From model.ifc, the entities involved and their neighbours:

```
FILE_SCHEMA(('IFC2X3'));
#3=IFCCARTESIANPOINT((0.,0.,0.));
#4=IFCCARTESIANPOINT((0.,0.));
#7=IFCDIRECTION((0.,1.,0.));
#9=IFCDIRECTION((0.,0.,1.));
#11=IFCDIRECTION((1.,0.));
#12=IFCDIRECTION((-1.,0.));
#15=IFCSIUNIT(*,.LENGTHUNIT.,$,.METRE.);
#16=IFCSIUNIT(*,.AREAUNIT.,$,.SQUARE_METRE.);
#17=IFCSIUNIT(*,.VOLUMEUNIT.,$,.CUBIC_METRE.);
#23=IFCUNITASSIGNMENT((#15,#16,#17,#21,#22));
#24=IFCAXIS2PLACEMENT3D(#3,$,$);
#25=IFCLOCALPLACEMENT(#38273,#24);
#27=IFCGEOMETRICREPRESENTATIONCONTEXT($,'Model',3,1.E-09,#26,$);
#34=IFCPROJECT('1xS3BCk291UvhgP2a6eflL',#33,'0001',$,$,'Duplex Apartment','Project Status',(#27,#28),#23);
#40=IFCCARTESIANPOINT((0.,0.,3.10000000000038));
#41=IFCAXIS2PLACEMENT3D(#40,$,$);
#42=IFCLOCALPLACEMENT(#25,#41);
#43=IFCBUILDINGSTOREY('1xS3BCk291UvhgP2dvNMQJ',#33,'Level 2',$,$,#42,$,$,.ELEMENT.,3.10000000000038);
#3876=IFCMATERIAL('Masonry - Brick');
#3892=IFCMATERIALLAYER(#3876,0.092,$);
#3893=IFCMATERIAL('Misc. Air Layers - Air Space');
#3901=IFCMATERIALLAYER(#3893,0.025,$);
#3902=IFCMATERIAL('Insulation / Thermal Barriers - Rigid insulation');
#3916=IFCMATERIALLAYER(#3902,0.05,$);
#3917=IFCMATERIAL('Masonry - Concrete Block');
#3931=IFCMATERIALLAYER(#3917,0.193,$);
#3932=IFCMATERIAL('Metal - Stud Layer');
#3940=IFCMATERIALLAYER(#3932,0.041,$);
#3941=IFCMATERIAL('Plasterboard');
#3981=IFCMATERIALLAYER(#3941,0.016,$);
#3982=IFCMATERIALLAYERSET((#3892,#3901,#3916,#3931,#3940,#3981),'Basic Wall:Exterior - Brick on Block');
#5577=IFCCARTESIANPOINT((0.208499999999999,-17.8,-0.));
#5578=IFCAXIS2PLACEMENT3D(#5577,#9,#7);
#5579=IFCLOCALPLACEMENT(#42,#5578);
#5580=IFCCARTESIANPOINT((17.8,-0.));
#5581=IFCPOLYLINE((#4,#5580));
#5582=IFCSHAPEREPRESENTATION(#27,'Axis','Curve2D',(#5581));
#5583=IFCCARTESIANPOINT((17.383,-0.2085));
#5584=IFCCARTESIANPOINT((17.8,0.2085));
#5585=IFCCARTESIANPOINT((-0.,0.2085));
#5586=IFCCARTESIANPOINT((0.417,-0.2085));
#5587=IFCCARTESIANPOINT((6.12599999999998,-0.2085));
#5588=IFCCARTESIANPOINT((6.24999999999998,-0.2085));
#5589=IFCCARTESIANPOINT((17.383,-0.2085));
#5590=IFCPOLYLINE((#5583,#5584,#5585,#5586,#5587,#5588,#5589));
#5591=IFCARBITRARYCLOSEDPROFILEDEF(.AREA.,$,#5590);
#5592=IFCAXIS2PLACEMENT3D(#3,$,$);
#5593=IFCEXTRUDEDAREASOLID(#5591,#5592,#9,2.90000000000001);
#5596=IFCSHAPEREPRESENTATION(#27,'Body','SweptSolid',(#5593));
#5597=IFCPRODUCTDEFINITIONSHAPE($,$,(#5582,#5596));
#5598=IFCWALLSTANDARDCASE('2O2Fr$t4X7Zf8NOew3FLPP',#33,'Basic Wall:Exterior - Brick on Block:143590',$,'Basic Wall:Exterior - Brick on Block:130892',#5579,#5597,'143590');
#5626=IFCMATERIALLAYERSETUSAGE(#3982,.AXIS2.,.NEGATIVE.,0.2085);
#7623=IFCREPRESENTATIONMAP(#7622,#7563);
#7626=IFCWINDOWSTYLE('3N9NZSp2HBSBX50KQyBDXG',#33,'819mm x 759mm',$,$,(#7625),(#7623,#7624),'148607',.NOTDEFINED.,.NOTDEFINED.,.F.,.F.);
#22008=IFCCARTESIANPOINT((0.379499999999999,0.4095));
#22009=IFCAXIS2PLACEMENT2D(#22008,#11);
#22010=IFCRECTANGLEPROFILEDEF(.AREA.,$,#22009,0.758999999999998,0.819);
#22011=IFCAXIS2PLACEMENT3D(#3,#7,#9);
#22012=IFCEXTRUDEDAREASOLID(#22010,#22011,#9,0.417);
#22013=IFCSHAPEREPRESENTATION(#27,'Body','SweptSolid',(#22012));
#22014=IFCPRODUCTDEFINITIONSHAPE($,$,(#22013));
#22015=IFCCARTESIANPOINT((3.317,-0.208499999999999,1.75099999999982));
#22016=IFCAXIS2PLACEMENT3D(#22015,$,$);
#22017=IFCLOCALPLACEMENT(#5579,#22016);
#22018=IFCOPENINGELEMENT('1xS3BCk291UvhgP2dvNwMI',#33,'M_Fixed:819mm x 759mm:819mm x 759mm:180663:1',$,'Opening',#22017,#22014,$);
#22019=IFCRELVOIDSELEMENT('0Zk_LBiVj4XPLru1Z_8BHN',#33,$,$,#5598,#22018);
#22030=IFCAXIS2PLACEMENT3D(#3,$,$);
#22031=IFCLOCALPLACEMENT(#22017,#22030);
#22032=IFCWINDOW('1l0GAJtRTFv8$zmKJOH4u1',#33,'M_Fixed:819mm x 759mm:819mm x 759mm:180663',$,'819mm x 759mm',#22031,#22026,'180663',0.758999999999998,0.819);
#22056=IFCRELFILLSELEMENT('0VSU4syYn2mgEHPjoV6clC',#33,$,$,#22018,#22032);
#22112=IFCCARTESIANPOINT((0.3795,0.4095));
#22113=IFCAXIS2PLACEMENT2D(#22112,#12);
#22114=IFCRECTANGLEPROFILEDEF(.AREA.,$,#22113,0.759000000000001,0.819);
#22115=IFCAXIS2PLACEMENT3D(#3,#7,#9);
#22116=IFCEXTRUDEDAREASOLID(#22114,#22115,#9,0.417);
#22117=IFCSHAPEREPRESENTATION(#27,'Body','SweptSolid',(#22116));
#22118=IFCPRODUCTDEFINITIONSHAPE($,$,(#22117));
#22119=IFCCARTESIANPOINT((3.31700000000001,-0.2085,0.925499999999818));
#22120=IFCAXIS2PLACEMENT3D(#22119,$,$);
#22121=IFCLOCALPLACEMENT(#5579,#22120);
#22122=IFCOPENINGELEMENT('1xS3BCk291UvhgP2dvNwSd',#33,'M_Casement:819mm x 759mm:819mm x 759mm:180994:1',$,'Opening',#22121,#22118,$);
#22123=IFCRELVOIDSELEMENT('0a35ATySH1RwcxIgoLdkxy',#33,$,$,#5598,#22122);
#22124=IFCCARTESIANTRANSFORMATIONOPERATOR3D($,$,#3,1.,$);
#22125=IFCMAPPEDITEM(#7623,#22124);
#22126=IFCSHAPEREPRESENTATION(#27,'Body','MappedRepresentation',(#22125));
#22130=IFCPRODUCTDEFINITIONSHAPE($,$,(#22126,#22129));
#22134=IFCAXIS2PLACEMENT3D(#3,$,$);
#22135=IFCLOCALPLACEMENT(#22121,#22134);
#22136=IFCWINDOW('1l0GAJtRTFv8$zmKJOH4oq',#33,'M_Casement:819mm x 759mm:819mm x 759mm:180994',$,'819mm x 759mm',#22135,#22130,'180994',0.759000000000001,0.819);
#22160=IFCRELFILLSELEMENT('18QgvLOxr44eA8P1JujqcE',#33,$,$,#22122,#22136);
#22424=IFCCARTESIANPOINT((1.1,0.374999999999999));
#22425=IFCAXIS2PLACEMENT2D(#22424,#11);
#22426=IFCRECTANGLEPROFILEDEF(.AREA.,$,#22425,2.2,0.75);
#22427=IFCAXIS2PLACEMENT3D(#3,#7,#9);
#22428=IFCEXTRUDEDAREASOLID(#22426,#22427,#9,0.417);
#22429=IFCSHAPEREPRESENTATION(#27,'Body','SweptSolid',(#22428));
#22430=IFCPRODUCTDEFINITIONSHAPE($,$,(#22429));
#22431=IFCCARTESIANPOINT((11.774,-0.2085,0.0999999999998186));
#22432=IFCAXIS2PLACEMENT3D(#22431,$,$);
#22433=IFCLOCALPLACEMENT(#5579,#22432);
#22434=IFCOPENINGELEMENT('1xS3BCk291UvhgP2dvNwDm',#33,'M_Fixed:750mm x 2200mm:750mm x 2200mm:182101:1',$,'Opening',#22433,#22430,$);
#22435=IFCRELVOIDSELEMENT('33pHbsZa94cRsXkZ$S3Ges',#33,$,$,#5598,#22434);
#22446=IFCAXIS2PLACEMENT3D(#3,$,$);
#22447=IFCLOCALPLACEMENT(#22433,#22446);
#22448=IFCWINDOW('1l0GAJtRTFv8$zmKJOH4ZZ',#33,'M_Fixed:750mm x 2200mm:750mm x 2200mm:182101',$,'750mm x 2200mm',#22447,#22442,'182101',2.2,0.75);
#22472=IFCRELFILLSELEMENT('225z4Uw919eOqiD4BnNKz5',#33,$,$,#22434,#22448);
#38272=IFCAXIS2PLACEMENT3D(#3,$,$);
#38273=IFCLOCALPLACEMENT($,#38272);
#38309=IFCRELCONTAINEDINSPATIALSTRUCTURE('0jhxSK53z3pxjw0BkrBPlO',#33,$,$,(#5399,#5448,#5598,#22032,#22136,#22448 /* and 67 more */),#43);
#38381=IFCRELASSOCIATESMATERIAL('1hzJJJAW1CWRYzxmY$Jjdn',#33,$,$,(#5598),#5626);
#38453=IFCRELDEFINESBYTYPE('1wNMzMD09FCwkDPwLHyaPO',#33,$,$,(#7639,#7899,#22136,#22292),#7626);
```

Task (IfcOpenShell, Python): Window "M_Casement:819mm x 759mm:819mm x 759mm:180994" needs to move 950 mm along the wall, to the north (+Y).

```python
import ifcopenshell
import ifcopenshell.api.geometry
import ifcopenshell.util.placement
import ifcopenshell.util.unit

model = ifcopenshell.open("model.ifc")
unit_scale = ifcopenshell.util.unit.calculate_unit_scale(model)

window = model.by_id(22136)
opening = window.FillsVoids[0].RelatingOpeningElement
wall = opening.VoidsElements[0].RelatingBuildingElement

wall_matrix = ifcopenshell.util.placement.get_local_placement(wall.ObjectPlacement)
shift = wall_matrix[:3, 0] * 0.95 / unit_scale
before = ifcopenshell.util.placement.get_local_placement(window.ObjectPlacement)[:3, 3].copy()

# The window is placed relative to its opening, so it follows when the opening moves.
matrix = ifcopenshell.util.placement.get_local_placement(opening.ObjectPlacement)
matrix[:3, 3] += shift
ifcopenshell.api.geometry.edit_object_placement(
    model, product=opening, matrix=matrix, is_si=False, should_transform_children=True
)

after = ifcopenshell.util.placement.get_local_placement(window.ObjectPlacement)[:3, 3]
print("window moved by", (after - before).round(3) + 0.0)

model.write("model_v2.ifc")
```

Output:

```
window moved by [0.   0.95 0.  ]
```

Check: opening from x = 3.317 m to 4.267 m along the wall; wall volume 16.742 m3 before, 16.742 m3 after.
